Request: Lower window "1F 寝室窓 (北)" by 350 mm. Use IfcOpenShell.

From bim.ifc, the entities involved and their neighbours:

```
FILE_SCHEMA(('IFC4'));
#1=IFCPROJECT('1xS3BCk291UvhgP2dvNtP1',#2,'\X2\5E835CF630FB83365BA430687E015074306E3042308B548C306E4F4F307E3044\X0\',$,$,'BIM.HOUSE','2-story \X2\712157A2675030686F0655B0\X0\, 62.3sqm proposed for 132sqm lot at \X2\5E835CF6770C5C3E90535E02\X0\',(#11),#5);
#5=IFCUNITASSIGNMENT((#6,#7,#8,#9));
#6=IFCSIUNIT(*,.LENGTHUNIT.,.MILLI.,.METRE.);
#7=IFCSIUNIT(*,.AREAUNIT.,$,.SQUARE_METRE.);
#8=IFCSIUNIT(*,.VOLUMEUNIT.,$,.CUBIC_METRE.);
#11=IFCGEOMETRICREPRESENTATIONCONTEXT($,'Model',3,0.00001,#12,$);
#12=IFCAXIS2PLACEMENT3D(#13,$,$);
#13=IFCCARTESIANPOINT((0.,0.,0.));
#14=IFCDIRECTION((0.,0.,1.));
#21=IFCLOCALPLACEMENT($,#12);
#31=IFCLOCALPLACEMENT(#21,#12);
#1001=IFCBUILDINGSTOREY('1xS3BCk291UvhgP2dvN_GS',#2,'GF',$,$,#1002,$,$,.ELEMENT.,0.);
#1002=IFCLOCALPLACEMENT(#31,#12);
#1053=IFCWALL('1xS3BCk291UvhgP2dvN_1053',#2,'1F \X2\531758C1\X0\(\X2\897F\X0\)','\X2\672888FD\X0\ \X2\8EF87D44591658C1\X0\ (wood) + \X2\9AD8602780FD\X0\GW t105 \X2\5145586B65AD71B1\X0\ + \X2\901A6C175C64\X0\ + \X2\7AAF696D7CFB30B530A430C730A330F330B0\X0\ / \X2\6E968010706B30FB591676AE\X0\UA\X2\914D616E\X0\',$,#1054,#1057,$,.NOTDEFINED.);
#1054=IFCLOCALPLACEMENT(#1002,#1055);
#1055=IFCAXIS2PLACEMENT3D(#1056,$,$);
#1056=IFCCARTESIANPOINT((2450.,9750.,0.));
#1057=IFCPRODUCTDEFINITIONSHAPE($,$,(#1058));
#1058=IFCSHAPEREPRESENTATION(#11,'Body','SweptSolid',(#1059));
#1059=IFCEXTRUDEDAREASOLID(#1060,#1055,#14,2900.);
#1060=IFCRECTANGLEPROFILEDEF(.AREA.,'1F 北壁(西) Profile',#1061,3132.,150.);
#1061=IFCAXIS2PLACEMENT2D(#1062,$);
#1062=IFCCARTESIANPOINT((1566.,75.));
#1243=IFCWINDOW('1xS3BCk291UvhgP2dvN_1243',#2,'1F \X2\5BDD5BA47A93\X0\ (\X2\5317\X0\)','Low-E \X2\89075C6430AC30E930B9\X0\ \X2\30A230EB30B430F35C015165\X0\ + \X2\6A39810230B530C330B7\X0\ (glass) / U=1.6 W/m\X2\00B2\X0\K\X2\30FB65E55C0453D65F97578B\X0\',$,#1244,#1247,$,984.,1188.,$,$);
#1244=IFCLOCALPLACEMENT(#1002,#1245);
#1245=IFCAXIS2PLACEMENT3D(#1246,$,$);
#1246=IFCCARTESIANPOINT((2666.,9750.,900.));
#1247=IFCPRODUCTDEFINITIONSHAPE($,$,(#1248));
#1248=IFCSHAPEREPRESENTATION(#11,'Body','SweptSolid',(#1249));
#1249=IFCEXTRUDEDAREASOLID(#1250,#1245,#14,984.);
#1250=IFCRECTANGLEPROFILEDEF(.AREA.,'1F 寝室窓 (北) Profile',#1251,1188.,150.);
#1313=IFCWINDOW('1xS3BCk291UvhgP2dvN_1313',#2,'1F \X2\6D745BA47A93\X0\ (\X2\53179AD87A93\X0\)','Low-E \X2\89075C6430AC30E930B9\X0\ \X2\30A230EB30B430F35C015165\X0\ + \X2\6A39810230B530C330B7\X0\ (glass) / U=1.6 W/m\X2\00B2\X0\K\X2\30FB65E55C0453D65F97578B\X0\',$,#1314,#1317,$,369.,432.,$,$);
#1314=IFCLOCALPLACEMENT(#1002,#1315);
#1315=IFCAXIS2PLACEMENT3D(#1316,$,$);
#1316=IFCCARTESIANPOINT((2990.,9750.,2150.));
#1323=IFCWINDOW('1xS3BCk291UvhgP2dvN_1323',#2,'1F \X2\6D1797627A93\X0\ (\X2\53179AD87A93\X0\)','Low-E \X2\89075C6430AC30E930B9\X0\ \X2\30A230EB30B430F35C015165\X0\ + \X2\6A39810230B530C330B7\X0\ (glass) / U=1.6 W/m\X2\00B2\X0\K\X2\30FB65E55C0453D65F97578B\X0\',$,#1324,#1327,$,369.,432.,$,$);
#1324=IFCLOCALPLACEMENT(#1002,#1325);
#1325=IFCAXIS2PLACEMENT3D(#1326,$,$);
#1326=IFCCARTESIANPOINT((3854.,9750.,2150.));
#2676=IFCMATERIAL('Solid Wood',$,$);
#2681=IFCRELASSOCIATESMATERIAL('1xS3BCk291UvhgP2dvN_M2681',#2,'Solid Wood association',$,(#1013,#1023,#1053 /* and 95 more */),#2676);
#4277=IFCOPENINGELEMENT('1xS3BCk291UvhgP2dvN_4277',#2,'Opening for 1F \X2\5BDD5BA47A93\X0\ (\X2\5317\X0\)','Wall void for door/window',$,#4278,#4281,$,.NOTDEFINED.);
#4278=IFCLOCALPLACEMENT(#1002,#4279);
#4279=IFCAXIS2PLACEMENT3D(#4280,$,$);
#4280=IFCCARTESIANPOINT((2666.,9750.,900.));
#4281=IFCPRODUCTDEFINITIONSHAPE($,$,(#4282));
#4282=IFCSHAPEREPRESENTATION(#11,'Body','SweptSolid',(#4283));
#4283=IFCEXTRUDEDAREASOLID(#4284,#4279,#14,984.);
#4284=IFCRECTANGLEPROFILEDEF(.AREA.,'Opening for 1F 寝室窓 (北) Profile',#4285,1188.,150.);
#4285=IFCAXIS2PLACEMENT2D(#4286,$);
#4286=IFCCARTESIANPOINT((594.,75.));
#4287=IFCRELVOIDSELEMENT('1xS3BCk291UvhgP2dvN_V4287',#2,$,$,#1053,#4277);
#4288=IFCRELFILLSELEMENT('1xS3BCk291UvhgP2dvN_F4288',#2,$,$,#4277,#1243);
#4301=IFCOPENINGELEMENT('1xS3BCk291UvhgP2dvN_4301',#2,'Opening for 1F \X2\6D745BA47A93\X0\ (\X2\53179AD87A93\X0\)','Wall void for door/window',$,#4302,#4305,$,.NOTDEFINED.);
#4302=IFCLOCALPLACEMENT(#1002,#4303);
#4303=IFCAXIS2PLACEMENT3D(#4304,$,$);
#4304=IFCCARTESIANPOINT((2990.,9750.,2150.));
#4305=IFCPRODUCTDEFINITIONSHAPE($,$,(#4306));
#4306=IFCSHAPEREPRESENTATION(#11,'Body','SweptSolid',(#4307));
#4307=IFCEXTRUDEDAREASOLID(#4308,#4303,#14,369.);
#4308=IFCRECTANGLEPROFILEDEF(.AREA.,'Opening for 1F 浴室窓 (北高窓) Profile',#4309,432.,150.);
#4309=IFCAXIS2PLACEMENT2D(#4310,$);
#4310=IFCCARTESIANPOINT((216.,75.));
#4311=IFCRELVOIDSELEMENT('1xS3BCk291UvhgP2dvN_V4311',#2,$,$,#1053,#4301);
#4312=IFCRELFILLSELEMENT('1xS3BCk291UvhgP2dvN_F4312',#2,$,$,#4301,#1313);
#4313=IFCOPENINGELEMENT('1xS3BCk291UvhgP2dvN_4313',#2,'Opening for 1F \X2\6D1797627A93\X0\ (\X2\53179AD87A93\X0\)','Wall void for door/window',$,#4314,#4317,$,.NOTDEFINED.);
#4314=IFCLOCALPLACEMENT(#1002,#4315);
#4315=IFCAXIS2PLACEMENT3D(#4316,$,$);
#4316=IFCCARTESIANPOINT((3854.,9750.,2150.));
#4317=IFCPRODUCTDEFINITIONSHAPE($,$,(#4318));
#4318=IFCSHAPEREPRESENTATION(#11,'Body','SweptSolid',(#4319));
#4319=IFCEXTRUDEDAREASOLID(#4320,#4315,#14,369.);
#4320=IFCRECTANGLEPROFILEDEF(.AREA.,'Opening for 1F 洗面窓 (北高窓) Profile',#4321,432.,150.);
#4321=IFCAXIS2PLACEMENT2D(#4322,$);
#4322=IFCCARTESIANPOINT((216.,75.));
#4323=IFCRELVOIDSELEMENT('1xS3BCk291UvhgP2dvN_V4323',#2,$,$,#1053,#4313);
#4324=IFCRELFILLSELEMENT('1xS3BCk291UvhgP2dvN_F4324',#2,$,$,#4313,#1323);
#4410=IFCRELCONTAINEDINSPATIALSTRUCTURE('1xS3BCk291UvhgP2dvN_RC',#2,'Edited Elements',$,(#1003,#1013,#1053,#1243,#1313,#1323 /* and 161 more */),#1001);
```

```python
import numpy as np
import ifcopenshell
import ifcopenshell.api.geometry
import ifcopenshell.util.placement
import ifcopenshell.util.unit

model = ifcopenshell.open("bim.ifc")
unit_scale = ifcopenshell.util.unit.calculate_unit_scale(model)

window = model.by_id(1243)
opening = window.FillsVoids[0].RelatingOpeningElement
dz = -0.35 / unit_scale

shift = np.array([0.0, 0.0, dz])
# The window is not placed relative to its opening, so move both.
for product in (opening, window):
    matrix = ifcopenshell.util.placement.get_local_placement(product.ObjectPlacement)
    matrix[:3, 3] += shift
    ifcopenshell.api.geometry.edit_object_placement(model, product=product, matrix=matrix, is_si=False)

print(f"moved by {dz * unit_scale:+.3f} m")

model.write("bim_v2.ifc")
```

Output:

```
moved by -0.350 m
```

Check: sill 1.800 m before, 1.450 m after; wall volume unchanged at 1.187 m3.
